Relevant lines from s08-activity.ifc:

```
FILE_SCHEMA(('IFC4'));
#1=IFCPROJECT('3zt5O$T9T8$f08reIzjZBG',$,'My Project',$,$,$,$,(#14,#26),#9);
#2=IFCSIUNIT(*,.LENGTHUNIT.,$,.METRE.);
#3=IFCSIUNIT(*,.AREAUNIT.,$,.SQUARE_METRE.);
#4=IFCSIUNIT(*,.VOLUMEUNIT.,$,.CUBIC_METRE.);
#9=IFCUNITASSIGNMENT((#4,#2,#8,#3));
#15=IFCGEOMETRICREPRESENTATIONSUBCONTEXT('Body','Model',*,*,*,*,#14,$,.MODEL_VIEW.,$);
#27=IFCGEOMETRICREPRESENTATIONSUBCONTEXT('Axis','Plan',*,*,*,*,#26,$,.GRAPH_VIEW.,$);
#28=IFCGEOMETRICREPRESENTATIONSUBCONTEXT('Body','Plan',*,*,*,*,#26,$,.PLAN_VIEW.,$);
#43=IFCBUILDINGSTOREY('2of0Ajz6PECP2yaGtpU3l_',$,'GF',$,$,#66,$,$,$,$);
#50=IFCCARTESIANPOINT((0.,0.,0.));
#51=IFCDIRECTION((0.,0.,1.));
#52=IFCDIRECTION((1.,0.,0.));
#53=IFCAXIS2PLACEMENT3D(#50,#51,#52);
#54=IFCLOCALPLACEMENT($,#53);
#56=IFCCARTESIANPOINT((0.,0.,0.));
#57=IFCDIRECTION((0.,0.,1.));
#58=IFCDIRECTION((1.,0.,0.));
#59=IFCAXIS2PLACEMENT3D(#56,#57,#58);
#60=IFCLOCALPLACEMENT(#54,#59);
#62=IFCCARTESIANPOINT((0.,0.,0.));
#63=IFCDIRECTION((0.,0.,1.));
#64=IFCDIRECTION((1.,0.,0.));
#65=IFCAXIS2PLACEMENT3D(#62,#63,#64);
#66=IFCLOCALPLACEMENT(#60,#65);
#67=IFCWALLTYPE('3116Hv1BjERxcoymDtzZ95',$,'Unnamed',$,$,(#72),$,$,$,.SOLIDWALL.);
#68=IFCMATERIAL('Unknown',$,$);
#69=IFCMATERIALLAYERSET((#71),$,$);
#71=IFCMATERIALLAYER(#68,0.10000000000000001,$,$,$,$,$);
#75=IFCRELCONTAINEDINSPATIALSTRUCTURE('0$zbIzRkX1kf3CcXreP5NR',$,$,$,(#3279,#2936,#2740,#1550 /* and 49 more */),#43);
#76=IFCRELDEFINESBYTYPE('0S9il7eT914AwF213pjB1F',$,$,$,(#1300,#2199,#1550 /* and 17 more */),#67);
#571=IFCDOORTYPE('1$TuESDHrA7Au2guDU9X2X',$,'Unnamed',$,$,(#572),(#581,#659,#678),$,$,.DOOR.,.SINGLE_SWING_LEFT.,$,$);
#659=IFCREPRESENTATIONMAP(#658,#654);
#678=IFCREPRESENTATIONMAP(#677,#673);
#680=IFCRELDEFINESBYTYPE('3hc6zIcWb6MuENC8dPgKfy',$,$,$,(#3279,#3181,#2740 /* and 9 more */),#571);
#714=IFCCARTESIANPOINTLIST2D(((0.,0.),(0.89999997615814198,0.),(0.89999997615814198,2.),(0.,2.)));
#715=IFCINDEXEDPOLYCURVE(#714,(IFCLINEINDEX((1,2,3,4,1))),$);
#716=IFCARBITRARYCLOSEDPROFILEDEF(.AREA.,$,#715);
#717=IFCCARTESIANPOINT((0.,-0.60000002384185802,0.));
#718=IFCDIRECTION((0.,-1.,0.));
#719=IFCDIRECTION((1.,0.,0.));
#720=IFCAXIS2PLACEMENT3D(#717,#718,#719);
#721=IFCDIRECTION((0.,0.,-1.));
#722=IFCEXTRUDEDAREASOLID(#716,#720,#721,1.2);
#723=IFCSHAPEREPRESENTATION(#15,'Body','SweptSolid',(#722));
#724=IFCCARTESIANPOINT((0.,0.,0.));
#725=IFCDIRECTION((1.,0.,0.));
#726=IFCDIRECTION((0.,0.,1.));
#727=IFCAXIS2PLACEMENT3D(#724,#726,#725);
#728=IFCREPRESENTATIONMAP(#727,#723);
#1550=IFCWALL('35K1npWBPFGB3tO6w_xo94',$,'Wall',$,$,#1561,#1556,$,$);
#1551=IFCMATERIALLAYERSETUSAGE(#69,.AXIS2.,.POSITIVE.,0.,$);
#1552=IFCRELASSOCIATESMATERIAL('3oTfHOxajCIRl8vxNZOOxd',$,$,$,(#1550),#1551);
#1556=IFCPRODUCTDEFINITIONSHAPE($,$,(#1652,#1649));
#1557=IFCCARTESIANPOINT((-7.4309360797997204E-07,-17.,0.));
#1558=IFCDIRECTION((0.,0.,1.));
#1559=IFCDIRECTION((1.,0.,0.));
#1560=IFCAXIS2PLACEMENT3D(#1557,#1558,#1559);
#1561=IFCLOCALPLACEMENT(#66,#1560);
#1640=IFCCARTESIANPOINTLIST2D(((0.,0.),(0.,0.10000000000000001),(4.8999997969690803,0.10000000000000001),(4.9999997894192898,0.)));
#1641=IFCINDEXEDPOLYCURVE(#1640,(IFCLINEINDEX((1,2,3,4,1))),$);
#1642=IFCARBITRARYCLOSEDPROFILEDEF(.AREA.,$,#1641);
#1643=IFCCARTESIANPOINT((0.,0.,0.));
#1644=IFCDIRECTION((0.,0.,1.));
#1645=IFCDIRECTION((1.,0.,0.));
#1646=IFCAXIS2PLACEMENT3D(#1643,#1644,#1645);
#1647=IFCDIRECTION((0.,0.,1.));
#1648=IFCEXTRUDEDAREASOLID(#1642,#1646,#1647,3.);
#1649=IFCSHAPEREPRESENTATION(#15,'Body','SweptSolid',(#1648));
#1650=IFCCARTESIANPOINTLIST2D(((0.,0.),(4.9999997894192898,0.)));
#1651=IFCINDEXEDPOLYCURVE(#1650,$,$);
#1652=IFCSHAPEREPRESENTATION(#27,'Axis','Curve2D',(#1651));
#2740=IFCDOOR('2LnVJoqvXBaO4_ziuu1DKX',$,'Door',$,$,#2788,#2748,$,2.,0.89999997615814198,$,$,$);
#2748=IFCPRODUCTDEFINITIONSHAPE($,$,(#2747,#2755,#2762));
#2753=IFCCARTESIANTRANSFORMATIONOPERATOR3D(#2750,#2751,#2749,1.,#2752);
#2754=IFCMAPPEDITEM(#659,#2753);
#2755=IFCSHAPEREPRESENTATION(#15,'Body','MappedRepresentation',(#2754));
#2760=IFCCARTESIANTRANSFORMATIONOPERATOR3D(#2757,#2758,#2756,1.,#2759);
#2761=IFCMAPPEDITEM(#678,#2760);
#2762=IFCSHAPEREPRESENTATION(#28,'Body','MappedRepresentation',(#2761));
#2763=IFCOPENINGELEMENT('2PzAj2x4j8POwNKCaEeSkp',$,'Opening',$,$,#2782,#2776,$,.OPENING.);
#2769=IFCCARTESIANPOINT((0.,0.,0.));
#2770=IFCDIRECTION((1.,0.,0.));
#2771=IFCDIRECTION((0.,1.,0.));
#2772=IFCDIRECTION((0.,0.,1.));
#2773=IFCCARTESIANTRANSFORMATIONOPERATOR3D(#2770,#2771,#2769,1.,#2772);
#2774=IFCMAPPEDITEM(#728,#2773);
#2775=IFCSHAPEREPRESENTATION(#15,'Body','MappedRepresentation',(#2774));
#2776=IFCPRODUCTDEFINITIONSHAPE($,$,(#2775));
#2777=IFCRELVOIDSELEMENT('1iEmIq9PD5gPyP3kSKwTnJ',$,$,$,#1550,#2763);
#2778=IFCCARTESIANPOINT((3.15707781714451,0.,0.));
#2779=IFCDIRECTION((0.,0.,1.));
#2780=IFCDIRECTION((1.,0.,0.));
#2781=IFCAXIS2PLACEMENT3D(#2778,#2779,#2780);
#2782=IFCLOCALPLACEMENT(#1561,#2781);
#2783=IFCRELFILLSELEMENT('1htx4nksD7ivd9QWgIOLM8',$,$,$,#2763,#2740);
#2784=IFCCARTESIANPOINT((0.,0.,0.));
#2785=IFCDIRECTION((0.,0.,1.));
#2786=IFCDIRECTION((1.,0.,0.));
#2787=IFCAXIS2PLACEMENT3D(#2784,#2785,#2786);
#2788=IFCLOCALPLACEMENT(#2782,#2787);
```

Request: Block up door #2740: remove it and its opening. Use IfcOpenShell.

```python
import ifcopenshell
import ifcopenshell.api.feature
import ifcopenshell.api.root
import ifcopenshell.geom
import ifcopenshell.util.shape

model = ifcopenshell.open("s08-activity.ifc")
settings = ifcopenshell.geom.settings()


def volume(element):
    """Net volume in cubic metres, openings subtracted."""
    shape = ifcopenshell.geom.create_shape(settings, element)
    return ifcopenshell.util.shape.get_volume(shape.geometry)


door = model.by_guid("2LnVJoqvXBaO4_ziuu1DKX")
opening = door.FillsVoids[0].RelatingOpeningElement
wall = opening.VoidsElements[0].RelatingBuildingElement
before = volume(wall)

ifcopenshell.api.root.remove_product(model, product=door)
ifcopenshell.api.feature.remove_feature(model, feature=opening)

after = volume(wall)

print(f"wall volume {before:.3f} -> {after:.3f} m3")

model.write("s08-activity_v2.ifc")
```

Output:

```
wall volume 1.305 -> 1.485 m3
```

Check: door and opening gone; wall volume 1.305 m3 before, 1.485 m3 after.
